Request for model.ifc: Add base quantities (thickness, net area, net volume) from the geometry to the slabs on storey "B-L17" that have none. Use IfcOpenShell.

First a look at what the model holds.

```python
import ifcopenshell
import ifcopenshell.util.element
import ifcopenshell.util.unit

model = ifcopenshell.open("model.ifc")
print(model.schema)
for unit_type in ("LENGTHUNIT", "AREAUNIT", "VOLUMEUNIT"):
    print(unit_type, ifcopenshell.util.unit.calculate_unit_scale(model, unit_type))
storey = next(s for s in model.by_type("IfcBuildingStorey") if s.Name == "B-L17")
slabs = [e for e in ifcopenshell.util.element.get_decomposition(storey) if e.is_a("IfcSlab")]
for e in sorted(slabs, key=lambda e: e.id()):
    print(e.id(), e.is_a(), e.Name, list(ifcopenshell.util.element.get_psets(e, qtos_only=True)), sep=" | ")
```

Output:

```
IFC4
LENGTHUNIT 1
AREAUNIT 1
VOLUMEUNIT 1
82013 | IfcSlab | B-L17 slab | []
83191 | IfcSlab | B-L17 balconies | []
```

```python
import ifcopenshell
import ifcopenshell.api.pset
import ifcopenshell.geom
import ifcopenshell.util.element
import ifcopenshell.util.shape
import ifcopenshell.util.unit

model = ifcopenshell.open("model.ifc")
unit_scale = ifcopenshell.util.unit.calculate_unit_scale(model)
area_scale = ifcopenshell.util.unit.calculate_unit_scale(model, "AREAUNIT")
volume_scale = ifcopenshell.util.unit.calculate_unit_scale(model, "VOLUMEUNIT")
settings = ifcopenshell.geom.settings()

storey = next(s for s in model.by_type("IfcBuildingStorey") if s.Name == "B-L17")
slabs = [e for e in ifcopenshell.util.element.get_decomposition(storey) if e.is_a("IfcSlab")]

for e in sorted(slabs, key=lambda e: e.id()):
    if ifcopenshell.util.element.get_psets(e, qtos_only=True, should_inherit=False):
        continue
    # Geometry comes back in metres, in the element's own axes.
    shape = ifcopenshell.geom.create_shape(settings, e)
    values = {
        "Width": ifcopenshell.util.shape.get_z(shape.geometry) / unit_scale,
        "NetArea": ifcopenshell.util.shape.get_footprint_area(shape.geometry) / area_scale,
        "NetVolume": ifcopenshell.util.shape.get_volume(shape.geometry) / volume_scale,
    }
    qto = ifcopenshell.api.pset.add_qto(model, product=e, name="Qto_SlabBaseQuantities")
    ifcopenshell.api.pset.edit_qto(model, qto=qto, properties=values)
    print(e.id(), {k: round(v, 3) for k, v in values.items()})

model.write("model-out.ifc")
```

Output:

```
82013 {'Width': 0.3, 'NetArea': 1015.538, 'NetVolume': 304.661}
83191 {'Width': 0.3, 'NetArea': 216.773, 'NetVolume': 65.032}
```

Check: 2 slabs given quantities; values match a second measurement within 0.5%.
